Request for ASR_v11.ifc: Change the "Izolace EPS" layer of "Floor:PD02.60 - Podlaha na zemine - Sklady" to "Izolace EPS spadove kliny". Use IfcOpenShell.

First a look at what the model holds.

```python
import ifcopenshell
import ifcopenshell.util.element

model = ifcopenshell.open("ASR_v11.ifc")
print(model.schema)
for layer_set in model.by_type("IfcMaterialLayerSet"):
    if layer_set.LayerSetName == "Floor:PD02.60 - Podlaha na zemine - Sklady":
        for layer in layer_set.MaterialLayers:
            print(layer.id(), layer.Material and layer.Material.Name, layer.LayerThickness, sep=" | ")
        print(len(ifcopenshell.util.element.get_elements_by_material(model, layer_set)), "elements and types use it")
print(sorted(m.Name for m in model.by_type("IfcMaterial") if m.Name)[:60])
```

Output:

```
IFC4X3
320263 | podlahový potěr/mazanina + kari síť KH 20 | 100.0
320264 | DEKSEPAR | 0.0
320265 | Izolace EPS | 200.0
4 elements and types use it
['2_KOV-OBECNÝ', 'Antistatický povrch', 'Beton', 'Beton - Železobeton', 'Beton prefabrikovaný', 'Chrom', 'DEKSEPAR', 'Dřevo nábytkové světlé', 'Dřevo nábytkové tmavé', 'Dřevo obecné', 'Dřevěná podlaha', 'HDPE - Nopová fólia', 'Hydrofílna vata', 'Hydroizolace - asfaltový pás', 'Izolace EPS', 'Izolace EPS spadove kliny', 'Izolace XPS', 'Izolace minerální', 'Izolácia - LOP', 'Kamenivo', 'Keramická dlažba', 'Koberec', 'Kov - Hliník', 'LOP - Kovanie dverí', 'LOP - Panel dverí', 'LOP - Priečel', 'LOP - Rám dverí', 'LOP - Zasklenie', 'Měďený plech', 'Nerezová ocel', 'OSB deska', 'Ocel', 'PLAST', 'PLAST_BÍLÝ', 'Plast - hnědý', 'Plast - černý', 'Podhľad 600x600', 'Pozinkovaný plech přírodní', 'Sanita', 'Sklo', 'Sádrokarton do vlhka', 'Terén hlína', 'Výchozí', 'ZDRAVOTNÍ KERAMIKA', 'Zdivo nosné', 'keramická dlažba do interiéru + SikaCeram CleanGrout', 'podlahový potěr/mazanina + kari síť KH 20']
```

```python
import ifcopenshell
import ifcopenshell.api.material

model = ifcopenshell.open("ASR_v11.ifc")

layer_set = next(s for s in model.by_type("IfcMaterialLayerSet") if s.LayerSetName == "Floor:PD02.60 - Podlaha na zemine - Sklady")
layer = next(l for l in layer_set.MaterialLayers if l.Material and l.Material.Name == "Izolace EPS")
material = next(m for m in model.by_type("IfcMaterial") if m.Name == "Izolace EPS spadove kliny")

# Point this one layer at the other material; renaming the old one would change it everywhere.
ifcopenshell.api.material.edit_layer(model, layer=layer, attributes={"Name": material.Name}, material=material)

print([l.Material.Name if l.Material else None for l in layer_set.MaterialLayers])

model.write("ASR_v11_v2.ifc")
```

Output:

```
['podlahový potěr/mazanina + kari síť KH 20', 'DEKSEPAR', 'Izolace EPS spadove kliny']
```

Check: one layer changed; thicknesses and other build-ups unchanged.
